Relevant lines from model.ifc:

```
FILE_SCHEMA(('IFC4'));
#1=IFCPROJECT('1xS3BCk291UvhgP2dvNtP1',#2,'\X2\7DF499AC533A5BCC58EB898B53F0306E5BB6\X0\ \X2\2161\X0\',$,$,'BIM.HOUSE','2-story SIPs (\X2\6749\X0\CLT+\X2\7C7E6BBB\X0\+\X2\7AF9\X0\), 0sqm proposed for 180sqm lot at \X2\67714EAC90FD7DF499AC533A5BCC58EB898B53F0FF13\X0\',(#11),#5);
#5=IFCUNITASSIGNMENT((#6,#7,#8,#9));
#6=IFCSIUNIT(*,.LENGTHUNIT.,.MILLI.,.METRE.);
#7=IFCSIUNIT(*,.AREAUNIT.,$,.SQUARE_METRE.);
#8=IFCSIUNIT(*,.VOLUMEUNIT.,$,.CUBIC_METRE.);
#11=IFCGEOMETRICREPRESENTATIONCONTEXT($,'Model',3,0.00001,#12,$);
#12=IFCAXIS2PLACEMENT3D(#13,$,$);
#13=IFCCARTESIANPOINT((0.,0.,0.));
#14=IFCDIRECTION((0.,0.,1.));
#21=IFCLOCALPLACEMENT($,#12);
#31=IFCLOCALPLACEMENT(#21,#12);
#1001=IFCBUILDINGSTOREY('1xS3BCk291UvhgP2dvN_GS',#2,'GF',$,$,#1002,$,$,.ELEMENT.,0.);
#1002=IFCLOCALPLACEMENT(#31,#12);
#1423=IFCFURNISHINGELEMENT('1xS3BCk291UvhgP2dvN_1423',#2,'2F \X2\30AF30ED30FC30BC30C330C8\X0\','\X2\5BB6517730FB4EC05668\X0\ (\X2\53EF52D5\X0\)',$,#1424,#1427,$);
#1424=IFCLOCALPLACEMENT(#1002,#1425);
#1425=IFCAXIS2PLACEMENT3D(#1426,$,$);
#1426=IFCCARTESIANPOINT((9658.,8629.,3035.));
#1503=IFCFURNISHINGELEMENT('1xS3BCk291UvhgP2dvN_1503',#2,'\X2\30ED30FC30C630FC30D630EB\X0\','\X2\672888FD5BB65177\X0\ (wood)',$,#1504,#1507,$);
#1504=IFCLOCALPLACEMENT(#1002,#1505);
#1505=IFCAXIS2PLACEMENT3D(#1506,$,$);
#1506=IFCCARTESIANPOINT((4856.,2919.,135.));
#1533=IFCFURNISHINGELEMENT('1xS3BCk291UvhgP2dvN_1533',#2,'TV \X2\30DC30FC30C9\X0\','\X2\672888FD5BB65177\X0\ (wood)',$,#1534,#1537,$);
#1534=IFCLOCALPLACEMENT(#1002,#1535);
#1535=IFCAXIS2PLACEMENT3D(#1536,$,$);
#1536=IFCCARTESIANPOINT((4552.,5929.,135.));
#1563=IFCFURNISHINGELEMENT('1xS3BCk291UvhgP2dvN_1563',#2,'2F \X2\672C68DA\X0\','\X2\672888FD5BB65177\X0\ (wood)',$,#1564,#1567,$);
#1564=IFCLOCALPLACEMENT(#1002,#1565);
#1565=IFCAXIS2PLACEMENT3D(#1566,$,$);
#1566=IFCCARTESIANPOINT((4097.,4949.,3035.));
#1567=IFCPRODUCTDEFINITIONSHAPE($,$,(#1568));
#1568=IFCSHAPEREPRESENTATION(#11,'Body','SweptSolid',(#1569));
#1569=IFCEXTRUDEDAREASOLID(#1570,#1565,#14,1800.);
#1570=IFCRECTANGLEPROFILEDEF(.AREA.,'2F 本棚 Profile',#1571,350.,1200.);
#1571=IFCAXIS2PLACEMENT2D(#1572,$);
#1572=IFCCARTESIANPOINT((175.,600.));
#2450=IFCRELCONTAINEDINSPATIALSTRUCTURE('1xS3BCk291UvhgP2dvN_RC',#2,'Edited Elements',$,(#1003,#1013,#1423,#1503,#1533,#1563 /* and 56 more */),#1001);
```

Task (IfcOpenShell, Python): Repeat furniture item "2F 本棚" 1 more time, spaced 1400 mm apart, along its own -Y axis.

```python
import ifcopenshell
import ifcopenshell.api.geometry
import ifcopenshell.api.root
import ifcopenshell.util.element
import ifcopenshell.util.placement

model = ifcopenshell.open("model.ifc")


def reuse_history(source, copy):
    """copy_class also copies each property set's owner history, people and application; keep the originals."""
    for rel in copy.IsDefinedBy:
        if rel.is_a("IfcRelDefinesByProperties") and (history := rel.RelatingPropertyDefinition.OwnerHistory):
            rel.RelatingPropertyDefinition.OwnerHistory = source.OwnerHistory
            ifcopenshell.util.element.remove_deep2(model, history)


source = model.by_id(1563)
base = ifcopenshell.util.placement.get_local_placement(source.ObjectPlacement)
step = -base[:3, 1] * 1400.0

for i in range(1, 2):
    copy = ifcopenshell.api.root.copy_class(model, product=source)
    copy.Representation = ifcopenshell.util.element.copy_deep(
        model, source.Representation, exclude=["IfcGeometricRepresentationContext", "IfcRepresentationMap"]
    )
    reuse_history(source, copy)
    matrix = base.copy()
    matrix[:3, 3] += i * step
    print("added at", matrix[:3, 3].round(3) + 0.0)
    ifcopenshell.api.geometry.edit_object_placement(model, product=copy, matrix=matrix, is_si=False)

model.write("model_rev.ifc")
```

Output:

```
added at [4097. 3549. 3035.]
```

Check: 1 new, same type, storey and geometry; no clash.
